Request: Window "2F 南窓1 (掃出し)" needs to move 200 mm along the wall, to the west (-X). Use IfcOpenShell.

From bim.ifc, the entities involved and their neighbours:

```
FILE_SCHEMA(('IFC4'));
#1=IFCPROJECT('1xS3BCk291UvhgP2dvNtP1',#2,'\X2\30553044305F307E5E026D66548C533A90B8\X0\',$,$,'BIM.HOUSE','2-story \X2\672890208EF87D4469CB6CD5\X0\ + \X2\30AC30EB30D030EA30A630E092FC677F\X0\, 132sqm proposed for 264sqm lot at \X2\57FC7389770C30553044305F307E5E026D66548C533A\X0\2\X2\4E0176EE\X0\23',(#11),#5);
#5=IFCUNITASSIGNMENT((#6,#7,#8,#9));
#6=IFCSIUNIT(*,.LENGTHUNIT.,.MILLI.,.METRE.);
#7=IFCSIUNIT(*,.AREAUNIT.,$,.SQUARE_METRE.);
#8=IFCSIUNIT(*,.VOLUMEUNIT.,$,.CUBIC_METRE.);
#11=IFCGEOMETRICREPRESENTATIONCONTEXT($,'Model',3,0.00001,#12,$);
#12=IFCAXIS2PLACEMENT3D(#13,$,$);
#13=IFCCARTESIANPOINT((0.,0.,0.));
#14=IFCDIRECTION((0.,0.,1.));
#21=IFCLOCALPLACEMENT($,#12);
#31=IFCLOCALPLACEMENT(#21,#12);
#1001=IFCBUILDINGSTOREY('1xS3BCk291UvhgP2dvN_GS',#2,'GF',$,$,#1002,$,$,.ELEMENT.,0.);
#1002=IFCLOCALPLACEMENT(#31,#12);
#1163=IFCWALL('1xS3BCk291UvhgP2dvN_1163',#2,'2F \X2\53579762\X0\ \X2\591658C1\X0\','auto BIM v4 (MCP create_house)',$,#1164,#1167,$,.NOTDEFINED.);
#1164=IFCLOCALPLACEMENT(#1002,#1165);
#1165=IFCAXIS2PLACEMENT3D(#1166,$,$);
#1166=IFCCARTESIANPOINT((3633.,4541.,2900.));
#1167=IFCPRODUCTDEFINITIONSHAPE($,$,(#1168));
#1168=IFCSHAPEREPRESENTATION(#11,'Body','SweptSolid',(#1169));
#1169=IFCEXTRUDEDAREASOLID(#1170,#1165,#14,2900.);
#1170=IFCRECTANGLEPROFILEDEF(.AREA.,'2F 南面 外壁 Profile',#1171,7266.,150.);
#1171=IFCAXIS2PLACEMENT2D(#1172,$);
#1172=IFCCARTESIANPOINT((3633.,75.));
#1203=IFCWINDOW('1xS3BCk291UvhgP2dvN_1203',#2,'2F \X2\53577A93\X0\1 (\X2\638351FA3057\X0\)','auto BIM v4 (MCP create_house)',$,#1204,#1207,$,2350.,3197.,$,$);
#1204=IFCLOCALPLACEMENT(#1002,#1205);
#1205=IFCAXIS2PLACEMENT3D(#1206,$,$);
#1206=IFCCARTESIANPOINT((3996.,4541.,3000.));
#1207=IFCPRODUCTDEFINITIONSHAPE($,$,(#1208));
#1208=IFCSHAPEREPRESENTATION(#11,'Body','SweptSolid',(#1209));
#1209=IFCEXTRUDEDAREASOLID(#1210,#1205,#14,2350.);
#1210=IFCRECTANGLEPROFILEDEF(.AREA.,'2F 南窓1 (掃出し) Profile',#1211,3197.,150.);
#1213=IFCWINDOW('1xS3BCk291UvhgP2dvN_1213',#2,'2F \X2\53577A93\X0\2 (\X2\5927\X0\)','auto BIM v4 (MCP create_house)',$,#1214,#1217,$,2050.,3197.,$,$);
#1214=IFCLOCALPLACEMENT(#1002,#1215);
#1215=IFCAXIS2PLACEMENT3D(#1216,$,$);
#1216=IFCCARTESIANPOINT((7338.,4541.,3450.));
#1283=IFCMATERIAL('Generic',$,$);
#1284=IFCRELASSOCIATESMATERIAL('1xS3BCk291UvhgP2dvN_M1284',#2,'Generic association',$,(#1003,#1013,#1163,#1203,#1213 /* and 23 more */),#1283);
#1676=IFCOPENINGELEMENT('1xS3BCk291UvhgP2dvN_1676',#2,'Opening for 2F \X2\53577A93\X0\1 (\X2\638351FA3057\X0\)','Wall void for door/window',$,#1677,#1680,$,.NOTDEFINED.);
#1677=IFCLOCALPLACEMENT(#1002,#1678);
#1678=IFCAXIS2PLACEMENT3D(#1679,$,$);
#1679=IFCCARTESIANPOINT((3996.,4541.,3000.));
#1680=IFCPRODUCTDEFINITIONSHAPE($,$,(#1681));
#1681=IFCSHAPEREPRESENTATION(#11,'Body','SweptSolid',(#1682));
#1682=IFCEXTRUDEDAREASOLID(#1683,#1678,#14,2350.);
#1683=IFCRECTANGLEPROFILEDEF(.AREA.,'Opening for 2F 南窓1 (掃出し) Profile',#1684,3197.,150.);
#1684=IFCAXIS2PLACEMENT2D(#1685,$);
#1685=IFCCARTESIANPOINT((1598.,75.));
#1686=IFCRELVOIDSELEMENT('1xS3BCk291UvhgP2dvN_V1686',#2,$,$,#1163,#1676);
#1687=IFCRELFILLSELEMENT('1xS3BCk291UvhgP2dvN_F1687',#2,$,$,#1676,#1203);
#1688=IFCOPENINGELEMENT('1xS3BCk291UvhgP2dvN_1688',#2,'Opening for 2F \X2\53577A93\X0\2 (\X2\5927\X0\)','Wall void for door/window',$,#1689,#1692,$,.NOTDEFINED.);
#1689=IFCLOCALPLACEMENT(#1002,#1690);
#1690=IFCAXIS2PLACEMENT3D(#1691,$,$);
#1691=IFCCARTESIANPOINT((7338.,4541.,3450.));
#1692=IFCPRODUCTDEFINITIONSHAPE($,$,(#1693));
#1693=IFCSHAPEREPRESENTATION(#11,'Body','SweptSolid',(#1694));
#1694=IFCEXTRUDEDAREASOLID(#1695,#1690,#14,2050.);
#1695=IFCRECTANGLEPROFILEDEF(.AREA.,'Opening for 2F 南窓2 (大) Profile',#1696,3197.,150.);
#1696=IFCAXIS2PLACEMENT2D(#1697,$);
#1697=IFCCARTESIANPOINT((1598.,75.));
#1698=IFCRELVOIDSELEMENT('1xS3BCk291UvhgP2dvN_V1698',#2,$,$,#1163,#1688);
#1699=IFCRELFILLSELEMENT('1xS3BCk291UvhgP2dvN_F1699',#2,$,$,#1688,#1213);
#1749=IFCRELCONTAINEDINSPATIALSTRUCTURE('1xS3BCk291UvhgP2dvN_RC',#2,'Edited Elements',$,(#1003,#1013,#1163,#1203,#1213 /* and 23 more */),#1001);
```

```python
import ifcopenshell
import ifcopenshell.api.geometry
import ifcopenshell.util.placement
import ifcopenshell.util.unit

model = ifcopenshell.open("bim.ifc")
unit_scale = ifcopenshell.util.unit.calculate_unit_scale(model)

window = model.by_guid("1xS3BCk291UvhgP2dvN_1203")
opening = window.FillsVoids[0].RelatingOpeningElement
wall = opening.VoidsElements[0].RelatingBuildingElement

wall_matrix = ifcopenshell.util.placement.get_local_placement(wall.ObjectPlacement)
shift = wall_matrix[:3, 0] * -0.2 / unit_scale
before = ifcopenshell.util.placement.get_local_placement(window.ObjectPlacement)[:3, 3].copy()

# The window is not placed relative to its opening, so move both.
for product in (opening, window):
    matrix = ifcopenshell.util.placement.get_local_placement(product.ObjectPlacement)
    matrix[:3, 3] += shift
    ifcopenshell.api.geometry.edit_object_placement(model, product=product, matrix=matrix, is_si=False)

after = ifcopenshell.util.placement.get_local_placement(window.ObjectPlacement)[:3, 3]
print("window moved by", (after - before).round(3) + 0.0)

model.write("bim_edited.ifc")
```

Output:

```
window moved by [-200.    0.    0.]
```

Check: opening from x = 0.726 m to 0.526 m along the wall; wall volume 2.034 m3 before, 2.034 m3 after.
